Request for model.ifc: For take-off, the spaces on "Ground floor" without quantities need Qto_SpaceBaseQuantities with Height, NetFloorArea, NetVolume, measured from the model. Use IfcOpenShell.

First a look at what the model holds.

```python
import ifcopenshell
import ifcopenshell.util.element
import ifcopenshell.util.unit

model = ifcopenshell.open("model.ifc")
print(model.schema)
for unit_type in ("LENGTHUNIT", "AREAUNIT", "VOLUMEUNIT"):
    print(unit_type, ifcopenshell.util.unit.calculate_unit_scale(model, unit_type))
storey = next(s for s in model.by_type("IfcBuildingStorey") if s.Name == "Ground floor")
spaces = [e for e in ifcopenshell.util.element.get_decomposition(storey) if e.is_a("IfcSpace")]
for e in sorted(spaces, key=lambda e: e.id()):
    print(e.id(), e.is_a(), e.Name, list(ifcopenshell.util.element.get_psets(e, qtos_only=True)), sep=" | ")
```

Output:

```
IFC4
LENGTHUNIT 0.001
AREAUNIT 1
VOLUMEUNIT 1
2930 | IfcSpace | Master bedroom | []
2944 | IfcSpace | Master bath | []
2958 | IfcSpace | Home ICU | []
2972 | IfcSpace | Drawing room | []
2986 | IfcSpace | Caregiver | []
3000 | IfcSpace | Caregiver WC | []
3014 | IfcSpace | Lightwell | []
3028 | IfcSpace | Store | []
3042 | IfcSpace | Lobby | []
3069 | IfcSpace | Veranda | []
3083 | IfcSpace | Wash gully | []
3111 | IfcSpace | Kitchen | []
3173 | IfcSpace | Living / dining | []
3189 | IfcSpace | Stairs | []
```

```python
import ifcopenshell
import ifcopenshell.api.pset
import ifcopenshell.geom
import ifcopenshell.util.element
import ifcopenshell.util.shape
import ifcopenshell.util.unit

model = ifcopenshell.open("model.ifc")
unit_scale = ifcopenshell.util.unit.calculate_unit_scale(model)
area_scale = ifcopenshell.util.unit.calculate_unit_scale(model, "AREAUNIT")
volume_scale = ifcopenshell.util.unit.calculate_unit_scale(model, "VOLUMEUNIT")
settings = ifcopenshell.geom.settings()

storey = next(s for s in model.by_type("IfcBuildingStorey") if s.Name == "Ground floor")
spaces = [e for e in ifcopenshell.util.element.get_decomposition(storey) if e.is_a("IfcSpace")]

for e in sorted(spaces, key=lambda e: e.id()):
    if ifcopenshell.util.element.get_psets(e, qtos_only=True, should_inherit=False):
        continue
    # Geometry comes back in metres, in the element's own axes.
    shape = ifcopenshell.geom.create_shape(settings, e)
    values = {
        "Height": ifcopenshell.util.shape.get_z(shape.geometry) / unit_scale,
        "NetFloorArea": ifcopenshell.util.shape.get_footprint_area(shape.geometry) / area_scale,
        "NetVolume": ifcopenshell.util.shape.get_volume(shape.geometry) / volume_scale,
    }
    qto = ifcopenshell.api.pset.add_qto(model, product=e, name="Qto_SpaceBaseQuantities")
    ifcopenshell.api.pset.edit_qto(model, qto=qto, properties=values)
    print(e.id(), {k: round(v, 3) for k, v in values.items()})

model.write("model_updated.ifc")
```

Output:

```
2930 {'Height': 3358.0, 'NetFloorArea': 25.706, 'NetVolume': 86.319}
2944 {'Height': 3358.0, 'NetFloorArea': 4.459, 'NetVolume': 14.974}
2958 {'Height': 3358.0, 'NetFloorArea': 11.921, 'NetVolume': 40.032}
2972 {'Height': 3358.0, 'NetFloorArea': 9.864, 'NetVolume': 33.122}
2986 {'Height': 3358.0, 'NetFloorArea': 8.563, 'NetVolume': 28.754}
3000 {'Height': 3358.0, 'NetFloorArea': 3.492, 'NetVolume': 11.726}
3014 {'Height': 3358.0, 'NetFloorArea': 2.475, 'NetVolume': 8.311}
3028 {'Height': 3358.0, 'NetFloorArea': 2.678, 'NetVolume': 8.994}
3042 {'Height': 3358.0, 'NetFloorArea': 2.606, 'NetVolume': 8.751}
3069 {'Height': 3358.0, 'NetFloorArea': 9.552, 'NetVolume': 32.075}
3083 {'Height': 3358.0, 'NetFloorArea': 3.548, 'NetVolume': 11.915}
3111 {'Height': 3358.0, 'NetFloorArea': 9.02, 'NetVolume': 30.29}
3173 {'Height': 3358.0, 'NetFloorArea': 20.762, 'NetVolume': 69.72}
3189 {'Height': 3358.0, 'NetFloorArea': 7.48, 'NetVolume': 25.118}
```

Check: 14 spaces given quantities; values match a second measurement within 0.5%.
